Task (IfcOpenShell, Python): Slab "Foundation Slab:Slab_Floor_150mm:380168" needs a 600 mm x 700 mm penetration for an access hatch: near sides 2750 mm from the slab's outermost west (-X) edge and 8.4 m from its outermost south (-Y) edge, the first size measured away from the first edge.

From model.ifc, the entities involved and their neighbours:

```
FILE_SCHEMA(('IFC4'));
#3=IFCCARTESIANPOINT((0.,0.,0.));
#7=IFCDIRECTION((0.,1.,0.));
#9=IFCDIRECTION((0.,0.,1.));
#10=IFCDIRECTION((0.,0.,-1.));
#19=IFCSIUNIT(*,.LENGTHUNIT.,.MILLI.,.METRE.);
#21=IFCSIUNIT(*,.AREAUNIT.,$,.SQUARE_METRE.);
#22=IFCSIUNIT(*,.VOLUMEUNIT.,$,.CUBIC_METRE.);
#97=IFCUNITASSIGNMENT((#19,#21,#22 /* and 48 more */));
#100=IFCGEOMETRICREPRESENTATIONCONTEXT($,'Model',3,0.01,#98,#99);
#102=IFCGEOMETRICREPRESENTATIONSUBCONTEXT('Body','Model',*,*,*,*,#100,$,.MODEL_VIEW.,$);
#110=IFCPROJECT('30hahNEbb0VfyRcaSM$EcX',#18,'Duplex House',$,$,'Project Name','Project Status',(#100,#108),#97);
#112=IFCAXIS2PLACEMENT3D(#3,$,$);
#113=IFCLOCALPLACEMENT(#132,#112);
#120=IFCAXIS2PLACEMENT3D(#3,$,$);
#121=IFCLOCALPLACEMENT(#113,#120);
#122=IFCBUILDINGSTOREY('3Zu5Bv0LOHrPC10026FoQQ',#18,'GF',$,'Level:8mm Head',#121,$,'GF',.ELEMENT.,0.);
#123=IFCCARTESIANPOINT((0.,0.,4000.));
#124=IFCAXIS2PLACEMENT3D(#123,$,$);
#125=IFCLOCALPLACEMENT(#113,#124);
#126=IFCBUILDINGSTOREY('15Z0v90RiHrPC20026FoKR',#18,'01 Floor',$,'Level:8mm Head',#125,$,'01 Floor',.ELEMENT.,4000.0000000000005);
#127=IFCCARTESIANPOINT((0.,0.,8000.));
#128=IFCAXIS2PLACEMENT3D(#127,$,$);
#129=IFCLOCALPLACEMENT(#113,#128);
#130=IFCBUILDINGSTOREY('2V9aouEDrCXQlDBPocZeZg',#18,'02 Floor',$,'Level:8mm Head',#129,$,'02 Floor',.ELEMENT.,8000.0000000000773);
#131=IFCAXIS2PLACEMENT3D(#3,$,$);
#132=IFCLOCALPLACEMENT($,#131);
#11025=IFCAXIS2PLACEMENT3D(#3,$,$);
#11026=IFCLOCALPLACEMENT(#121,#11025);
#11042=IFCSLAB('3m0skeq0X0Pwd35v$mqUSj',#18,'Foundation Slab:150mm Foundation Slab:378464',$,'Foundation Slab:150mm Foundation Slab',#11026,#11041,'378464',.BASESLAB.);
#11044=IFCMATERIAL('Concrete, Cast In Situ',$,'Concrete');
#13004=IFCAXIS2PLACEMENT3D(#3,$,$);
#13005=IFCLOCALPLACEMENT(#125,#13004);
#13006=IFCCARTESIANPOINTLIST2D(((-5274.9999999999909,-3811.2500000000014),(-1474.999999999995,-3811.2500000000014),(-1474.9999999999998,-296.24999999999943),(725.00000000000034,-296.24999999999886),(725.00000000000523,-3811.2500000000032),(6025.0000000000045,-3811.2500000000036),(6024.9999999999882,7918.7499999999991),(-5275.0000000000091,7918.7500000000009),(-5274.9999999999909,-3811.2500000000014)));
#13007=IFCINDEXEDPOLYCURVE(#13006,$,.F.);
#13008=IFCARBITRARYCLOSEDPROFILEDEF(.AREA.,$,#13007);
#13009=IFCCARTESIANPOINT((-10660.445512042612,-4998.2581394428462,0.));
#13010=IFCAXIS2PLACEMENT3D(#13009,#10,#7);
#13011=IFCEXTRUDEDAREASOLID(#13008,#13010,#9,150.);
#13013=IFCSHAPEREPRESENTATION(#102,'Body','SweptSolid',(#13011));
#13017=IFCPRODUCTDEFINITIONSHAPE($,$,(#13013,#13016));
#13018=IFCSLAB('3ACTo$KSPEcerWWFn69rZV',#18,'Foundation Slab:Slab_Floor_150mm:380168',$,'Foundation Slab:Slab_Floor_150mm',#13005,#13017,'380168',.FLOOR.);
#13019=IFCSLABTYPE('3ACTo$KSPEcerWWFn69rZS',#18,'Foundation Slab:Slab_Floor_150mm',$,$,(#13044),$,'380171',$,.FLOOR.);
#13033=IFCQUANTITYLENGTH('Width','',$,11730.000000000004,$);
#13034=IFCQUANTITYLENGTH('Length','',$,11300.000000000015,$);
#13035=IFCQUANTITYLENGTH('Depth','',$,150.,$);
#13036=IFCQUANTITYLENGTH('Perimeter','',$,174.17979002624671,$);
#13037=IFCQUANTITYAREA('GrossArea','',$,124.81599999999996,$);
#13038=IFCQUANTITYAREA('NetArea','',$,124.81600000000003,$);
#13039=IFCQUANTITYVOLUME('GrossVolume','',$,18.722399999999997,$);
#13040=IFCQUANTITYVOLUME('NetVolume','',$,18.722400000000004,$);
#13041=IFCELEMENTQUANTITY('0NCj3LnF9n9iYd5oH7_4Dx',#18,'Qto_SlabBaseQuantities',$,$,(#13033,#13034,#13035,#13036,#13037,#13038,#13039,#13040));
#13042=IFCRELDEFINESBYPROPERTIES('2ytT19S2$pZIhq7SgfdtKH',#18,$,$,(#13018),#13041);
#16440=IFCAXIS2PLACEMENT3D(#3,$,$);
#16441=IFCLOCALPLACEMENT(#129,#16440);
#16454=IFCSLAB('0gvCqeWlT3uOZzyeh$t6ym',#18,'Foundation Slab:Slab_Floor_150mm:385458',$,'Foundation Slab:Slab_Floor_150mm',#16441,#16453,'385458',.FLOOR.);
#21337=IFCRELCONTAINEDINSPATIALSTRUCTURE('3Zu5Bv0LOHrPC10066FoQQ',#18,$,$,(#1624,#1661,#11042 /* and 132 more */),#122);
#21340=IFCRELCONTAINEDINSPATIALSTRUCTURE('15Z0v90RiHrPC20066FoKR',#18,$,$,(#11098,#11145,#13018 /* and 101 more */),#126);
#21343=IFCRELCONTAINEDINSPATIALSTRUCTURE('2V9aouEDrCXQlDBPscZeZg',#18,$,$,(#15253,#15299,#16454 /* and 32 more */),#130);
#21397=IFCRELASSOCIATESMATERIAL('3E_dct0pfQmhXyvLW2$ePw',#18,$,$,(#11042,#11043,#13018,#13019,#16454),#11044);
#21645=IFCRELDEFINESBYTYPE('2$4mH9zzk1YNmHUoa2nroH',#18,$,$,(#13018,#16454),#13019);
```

```python
import numpy as np
import ifcopenshell
import ifcopenshell.api.feature
import ifcopenshell.api.geometry
import ifcopenshell.api.pset
import ifcopenshell.api.root
import ifcopenshell.geom
import ifcopenshell.util.element
import ifcopenshell.util.placement
import ifcopenshell.util.representation
import ifcopenshell.util.shape
import ifcopenshell.util.unit

model = ifcopenshell.open("model.ifc")
unit_scale = ifcopenshell.util.unit.calculate_unit_scale(model)
area_scale = ifcopenshell.util.unit.calculate_unit_scale(model, "AREAUNIT")
volume_scale = ifcopenshell.util.unit.calculate_unit_scale(model, "VOLUMEUNIT")
settings = ifcopenshell.geom.settings()


def volume(element):
    """Net volume in cubic metres, openings subtracted."""
    shape = ifcopenshell.geom.create_shape(settings, element)
    return ifcopenshell.util.shape.get_volume(shape.geometry)


slab = model.by_guid("3ACTo$KSPEcerWWFn69rZV")
before = volume(slab)

# Extent in the slab's own axes, in metres. The edges named are its -X and -Y sides.
slab_shape = ifcopenshell.geom.create_shape(settings, slab)
vertices = ifcopenshell.util.shape.get_vertices(slab_shape.geometry)
x_min, y_min, bottom = vertices.min(axis=0)
top = vertices[:, 2].max()

opening = ifcopenshell.api.root.create_entity(model, ifc_class="IfcOpeningElement", name="Access hatch opening", predefined_type="OPENING")
context = ifcopenshell.util.representation.get_context(model, "Model", "Body", "MODEL_VIEW")
width, depth = 0.6, 0.7
outline = [(0.0, 0.0), (width, 0.0), (width, depth), (0.0, depth), (0.0, 0.0)]
# Overshoot both faces by 50 mm so the cut is clean.
shape = ifcopenshell.api.geometry.add_slab_representation(
    model, context=context, depth=top - bottom + 0.1, polyline=outline
)
ifcopenshell.api.geometry.assign_representation(model, product=opening, representation=shape)

matrix = ifcopenshell.util.placement.get_local_placement(slab.ObjectPlacement)
matrix[:, 3] = matrix @ np.append(np.array([x_min + 2.75, y_min + 8.4, bottom - 0.05]) / unit_scale, 1.0)
ifcopenshell.api.geometry.edit_object_placement(model, product=opening, matrix=matrix, is_si=False)
ifcopenshell.api.feature.add_feature(model, feature=opening, element=slab)

after = volume(slab)

# Update the slab's stored quantities.
qto = model.by_id(ifcopenshell.util.element.get_pset(slab, "Qto_SlabBaseQuantities", should_inherit=False)["id"])
ifcopenshell.api.pset.edit_qto(model, qto=qto, properties={
    "NetArea": after / (top - bottom) / area_scale,
    "NetVolume": after / volume_scale,
})

print(f"slab volume {before:.3f} -> {after:.3f} m3")

model.write("model-out.ifc")
```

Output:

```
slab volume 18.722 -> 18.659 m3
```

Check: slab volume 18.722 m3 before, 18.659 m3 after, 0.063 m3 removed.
